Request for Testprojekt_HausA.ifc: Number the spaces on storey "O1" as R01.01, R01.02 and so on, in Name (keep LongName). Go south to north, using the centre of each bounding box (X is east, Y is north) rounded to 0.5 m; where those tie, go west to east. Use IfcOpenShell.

First a look at what the model holds.

```python
import ifcopenshell
import ifcopenshell.util.element
import ifcopenshell.util.placement

model = ifcopenshell.open("Testprojekt_HausA.ifc")
print(model.schema)
storey = next(s for s in model.by_type("IfcBuildingStorey") if s.Name == "O1")
spaces = [e for e in ifcopenshell.util.element.get_decomposition(storey) if e.is_a("IfcSpace")]
for e in sorted(spaces, key=lambda e: e.id()):
    origin = ifcopenshell.util.placement.get_local_placement(e.ObjectPlacement)[:3, 3]
    print(e.id(), e.Name, e.LongName, origin.round(2) + 0.0, sep=" | ")
```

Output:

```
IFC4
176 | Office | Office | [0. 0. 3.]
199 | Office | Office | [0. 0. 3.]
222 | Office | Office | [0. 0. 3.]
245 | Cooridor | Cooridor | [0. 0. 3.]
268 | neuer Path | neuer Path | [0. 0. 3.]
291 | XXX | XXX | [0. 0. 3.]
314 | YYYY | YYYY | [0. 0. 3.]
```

```python
import ifcopenshell
import ifcopenshell.geom
import ifcopenshell.util.element
import ifcopenshell.util.shape

model = ifcopenshell.open("Testprojekt_HausA.ifc")
settings = ifcopenshell.geom.settings()
settings.set("use-world-coords", True)


def centre(element):
    shape = ifcopenshell.geom.create_shape(settings, element)
    return ifcopenshell.util.shape.get_bbox_centroid(shape.geometry)


storey = next(s for s in model.by_type("IfcBuildingStorey") if s.Name == "O1")
spaces = [e for e in ifcopenshell.util.element.get_decomposition(storey) if e.is_a("IfcSpace")]

# Insertion points can sit at a corner or the storey origin, so sort by the geometry (in metres).
centres = {e: centre(e) for e in spaces}
spaces.sort(key=lambda e: (round(centres[e][1] / 0.5), centres[e][0]))

for i, e in enumerate(spaces, start=1):
    number = f"R01.{i:02d}"
    e.Name = number
    print(e.id(), number)

model.write("Testprojekt_HausA_v2.ifc")
```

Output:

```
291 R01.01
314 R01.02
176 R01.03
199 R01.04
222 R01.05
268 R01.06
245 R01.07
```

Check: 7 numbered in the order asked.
